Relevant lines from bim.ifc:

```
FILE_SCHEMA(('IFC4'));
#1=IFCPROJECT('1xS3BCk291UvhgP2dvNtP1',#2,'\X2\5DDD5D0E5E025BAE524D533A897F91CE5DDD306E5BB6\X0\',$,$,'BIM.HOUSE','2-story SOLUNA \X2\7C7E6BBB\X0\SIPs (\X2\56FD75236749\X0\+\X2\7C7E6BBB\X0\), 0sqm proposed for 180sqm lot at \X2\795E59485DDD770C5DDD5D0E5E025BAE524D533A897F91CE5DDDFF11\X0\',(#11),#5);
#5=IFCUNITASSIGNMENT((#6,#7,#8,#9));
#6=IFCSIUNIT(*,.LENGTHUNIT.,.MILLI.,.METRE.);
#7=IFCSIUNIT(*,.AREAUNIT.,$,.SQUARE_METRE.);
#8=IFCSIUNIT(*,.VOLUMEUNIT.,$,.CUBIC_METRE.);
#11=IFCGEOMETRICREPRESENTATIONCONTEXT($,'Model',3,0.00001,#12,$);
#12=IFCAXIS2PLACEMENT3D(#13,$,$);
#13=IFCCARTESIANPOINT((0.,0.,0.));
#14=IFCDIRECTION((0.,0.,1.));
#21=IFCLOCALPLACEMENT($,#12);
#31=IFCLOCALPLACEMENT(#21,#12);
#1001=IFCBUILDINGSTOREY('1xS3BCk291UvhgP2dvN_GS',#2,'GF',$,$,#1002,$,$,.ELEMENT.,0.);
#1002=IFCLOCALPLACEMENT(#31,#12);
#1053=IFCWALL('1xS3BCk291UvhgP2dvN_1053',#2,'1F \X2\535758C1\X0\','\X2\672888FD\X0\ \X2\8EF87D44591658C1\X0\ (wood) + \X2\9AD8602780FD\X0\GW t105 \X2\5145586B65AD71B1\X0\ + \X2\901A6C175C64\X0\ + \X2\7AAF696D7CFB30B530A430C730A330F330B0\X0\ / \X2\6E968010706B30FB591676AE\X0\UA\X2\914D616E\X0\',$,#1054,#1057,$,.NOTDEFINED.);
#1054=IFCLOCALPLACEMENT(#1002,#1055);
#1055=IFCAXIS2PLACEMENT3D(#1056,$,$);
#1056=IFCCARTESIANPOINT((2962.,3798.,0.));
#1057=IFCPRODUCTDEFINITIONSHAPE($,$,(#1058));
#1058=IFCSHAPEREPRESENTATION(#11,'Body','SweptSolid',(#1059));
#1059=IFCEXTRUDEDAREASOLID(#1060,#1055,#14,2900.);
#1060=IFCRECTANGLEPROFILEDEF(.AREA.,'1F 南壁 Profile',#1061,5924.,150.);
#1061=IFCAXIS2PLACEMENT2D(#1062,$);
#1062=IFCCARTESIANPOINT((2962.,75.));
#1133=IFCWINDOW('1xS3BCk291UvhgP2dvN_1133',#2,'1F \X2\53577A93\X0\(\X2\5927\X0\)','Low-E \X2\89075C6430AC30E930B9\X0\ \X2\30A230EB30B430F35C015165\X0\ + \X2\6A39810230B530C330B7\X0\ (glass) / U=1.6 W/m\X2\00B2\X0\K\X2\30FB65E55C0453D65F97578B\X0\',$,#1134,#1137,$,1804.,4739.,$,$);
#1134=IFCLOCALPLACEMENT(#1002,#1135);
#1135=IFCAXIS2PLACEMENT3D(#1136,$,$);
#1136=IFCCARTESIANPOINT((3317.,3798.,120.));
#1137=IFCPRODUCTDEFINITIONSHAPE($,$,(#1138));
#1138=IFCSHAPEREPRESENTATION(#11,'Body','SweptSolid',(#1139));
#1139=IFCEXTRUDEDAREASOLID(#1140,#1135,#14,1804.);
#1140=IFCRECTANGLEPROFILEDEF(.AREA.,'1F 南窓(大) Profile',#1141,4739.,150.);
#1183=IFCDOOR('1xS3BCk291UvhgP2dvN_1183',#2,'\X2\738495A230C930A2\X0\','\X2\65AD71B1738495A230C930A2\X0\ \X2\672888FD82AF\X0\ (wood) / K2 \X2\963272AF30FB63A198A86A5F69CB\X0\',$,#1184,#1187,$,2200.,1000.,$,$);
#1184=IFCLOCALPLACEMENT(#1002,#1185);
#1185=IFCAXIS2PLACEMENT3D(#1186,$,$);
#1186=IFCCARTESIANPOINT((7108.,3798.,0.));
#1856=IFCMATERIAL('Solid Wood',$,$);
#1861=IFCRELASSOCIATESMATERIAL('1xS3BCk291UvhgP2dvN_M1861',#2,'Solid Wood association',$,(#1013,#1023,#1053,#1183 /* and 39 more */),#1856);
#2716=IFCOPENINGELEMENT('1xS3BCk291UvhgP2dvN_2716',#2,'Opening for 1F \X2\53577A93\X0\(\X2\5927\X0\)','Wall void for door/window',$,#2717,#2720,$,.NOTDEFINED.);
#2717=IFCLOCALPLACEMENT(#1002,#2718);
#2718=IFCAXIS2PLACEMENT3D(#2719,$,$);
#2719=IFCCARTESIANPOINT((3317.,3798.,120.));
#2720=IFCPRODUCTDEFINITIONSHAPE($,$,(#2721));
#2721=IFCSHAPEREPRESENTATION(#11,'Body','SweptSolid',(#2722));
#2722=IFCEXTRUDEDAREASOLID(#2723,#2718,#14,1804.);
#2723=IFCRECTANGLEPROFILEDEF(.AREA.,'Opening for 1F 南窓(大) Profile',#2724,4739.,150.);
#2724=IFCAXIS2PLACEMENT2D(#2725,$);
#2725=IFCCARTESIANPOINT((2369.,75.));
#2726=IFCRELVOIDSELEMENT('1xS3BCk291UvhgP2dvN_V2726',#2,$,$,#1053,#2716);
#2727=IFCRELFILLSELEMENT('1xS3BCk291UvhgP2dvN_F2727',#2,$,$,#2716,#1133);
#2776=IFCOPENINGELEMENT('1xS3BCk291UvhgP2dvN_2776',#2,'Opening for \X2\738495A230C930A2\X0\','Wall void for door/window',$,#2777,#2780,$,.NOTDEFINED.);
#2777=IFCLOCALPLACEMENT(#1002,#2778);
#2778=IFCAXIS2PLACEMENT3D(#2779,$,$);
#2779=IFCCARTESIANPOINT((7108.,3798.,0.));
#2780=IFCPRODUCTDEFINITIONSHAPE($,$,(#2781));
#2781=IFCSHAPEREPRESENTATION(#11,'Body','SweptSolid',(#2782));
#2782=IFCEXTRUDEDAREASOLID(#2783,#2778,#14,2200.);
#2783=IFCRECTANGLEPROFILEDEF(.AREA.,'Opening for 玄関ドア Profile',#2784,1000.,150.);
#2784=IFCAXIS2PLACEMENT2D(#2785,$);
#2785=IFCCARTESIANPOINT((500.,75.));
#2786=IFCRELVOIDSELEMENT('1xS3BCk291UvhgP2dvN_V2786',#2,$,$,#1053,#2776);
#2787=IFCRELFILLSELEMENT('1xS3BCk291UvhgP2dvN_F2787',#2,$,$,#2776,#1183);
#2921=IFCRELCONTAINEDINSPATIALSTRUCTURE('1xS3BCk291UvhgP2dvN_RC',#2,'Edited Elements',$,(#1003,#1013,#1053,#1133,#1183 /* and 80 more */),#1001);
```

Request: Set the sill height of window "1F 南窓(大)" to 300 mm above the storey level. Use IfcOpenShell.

```python
import numpy as np
import ifcopenshell
import ifcopenshell.api.geometry
import ifcopenshell.geom
import ifcopenshell.util.element
import ifcopenshell.util.placement
import ifcopenshell.util.shape
import ifcopenshell.util.unit

model = ifcopenshell.open("bim.ifc")
unit_scale = ifcopenshell.util.unit.calculate_unit_scale(model)

window = model.by_guid("1xS3BCk291UvhgP2dvN_1133")
opening = window.FillsVoids[0].RelatingOpeningElement
storey = ifcopenshell.util.element.get_container(window, ifc_class="IfcBuildingStorey")
level = ifcopenshell.util.placement.get_local_placement(storey.ObjectPlacement)[2, 3]

# The opening's origin need not be at the sill, so measure its lowest point.
shape = ifcopenshell.geom.create_shape(ifcopenshell.geom.settings(), opening)
bottom = ifcopenshell.util.shape.get_shape_bottom_elevation(shape, shape.geometry) / unit_scale
dz = level + 0.3 / unit_scale - bottom

shift = np.array([0.0, 0.0, dz])
# The window is not placed relative to its opening, so move both.
for product in (opening, window):
    matrix = ifcopenshell.util.placement.get_local_placement(product.ObjectPlacement)
    matrix[:3, 3] += shift
    ifcopenshell.api.geometry.edit_object_placement(model, product=product, matrix=matrix, is_si=False)

print(f"moved by {dz * unit_scale:+.3f} m")

model.write("bim_v2.ifc")
```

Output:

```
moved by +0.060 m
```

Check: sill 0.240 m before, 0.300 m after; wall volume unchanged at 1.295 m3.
